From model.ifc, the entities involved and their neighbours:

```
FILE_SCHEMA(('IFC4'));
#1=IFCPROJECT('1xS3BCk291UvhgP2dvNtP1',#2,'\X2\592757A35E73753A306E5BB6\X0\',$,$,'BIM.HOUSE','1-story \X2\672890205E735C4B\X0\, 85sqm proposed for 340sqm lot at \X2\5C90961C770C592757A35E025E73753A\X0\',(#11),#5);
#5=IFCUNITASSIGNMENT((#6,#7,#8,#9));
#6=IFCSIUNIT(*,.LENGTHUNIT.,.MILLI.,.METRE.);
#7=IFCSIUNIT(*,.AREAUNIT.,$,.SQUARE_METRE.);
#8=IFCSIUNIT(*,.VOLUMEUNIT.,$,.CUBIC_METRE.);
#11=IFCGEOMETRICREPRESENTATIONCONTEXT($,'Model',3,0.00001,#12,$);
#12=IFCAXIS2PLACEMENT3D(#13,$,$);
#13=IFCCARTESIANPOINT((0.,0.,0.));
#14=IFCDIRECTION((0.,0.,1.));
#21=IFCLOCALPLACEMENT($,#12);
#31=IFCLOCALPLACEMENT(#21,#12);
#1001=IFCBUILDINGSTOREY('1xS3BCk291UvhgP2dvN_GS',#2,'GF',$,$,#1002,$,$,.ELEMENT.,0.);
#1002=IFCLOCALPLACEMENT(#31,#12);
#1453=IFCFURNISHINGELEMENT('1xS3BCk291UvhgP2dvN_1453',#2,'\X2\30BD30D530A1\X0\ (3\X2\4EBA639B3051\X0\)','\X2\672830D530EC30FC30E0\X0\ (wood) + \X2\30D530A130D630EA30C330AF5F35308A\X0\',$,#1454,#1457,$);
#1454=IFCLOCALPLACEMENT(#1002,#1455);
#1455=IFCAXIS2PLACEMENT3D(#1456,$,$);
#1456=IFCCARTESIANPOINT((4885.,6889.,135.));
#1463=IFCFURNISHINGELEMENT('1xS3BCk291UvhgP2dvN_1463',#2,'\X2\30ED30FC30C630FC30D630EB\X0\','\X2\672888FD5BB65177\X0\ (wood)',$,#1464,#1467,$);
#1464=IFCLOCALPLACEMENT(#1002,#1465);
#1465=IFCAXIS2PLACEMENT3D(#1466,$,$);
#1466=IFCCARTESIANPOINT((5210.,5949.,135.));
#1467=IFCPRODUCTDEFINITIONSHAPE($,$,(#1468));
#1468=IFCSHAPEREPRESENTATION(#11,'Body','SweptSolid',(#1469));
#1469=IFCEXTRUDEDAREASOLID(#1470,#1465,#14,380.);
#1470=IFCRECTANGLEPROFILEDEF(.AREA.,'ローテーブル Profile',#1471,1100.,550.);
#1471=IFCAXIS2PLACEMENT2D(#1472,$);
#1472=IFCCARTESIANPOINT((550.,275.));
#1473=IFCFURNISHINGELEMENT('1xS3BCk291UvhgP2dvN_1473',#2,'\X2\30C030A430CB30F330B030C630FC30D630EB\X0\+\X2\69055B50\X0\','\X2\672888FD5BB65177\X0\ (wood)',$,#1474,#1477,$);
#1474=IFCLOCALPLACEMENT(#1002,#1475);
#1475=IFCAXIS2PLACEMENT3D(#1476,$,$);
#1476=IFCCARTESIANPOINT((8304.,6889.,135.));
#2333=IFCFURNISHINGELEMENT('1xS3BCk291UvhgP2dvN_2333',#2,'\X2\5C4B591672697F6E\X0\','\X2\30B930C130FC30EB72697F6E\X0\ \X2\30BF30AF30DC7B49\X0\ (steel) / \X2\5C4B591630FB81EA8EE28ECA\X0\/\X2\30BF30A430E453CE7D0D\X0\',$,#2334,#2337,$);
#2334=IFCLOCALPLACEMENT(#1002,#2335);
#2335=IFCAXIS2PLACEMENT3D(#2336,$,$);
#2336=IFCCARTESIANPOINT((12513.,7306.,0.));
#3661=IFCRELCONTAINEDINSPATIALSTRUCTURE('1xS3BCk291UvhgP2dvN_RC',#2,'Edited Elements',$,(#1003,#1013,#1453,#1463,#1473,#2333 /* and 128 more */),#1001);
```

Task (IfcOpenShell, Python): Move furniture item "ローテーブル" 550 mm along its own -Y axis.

```python
import ifcopenshell
import ifcopenshell.api.geometry
import ifcopenshell.util.placement
import ifcopenshell.util.unit

model = ifcopenshell.open("model.ifc")
unit_scale = ifcopenshell.util.unit.calculate_unit_scale(model)

item = model.by_guid("1xS3BCk291UvhgP2dvN_1463")
matrix = ifcopenshell.util.placement.get_local_placement(item.ObjectPlacement)
matrix[:3, 3] -= matrix[:3, 1] * 0.55 / unit_scale
ifcopenshell.api.geometry.edit_object_placement(model, product=item, matrix=matrix, is_si=False)

print(ifcopenshell.util.placement.get_local_placement(item.ObjectPlacement).round(3) + 0.0)

model.write("model_updated.ifc")
```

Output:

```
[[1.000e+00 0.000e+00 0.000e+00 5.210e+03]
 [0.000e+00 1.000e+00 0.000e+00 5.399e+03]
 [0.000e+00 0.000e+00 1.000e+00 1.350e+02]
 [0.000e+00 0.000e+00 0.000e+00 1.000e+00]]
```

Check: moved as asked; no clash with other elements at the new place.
